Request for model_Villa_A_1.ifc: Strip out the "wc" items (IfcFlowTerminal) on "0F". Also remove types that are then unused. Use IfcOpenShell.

First a look at what the model holds.

```python
import ifcopenshell
import ifcopenshell.util.element

model = ifcopenshell.open("model_Villa_A_1.ifc")
print(model.schema)
storey = next(s for s in model.by_type("IfcBuildingStorey") if s.Name == "0F")
terminals = [e for e in ifcopenshell.util.element.get_decomposition(storey) if e.is_a("IfcFlowTerminal")]
seen = {}
for e in terminals:
    element_type = ifcopenshell.util.element.get_type(e)
    name = element_type.Name if element_type not in (None, e) else None
    seen[name] = seen.get(name, 0) + 1
for name, count in sorted(seen.items(), key=str):
    print(count, "x", name)
```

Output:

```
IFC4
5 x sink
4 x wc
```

```python
import ifcopenshell
import ifcopenshell.api.root
import ifcopenshell.util.element

model = ifcopenshell.open("model_Villa_A_1.ifc")

storey = next(s for s in model.by_type("IfcBuildingStorey") if s.Name == "0F")
terminals = [e for e in ifcopenshell.util.element.get_decomposition(storey) if e.is_a("IfcFlowTerminal")]
targets = [e for e in terminals if (t := ifcopenshell.util.element.get_type(e)) not in (None, e) and t.Name == "wc"]
types = {ifcopenshell.util.element.get_type(e) for e in targets} - {None, *targets}

for e in targets:
    ifcopenshell.api.root.remove_product(model, product=e)
print(len(targets), "removed")

unused = [t for t in types if not ifcopenshell.util.element.get_types(t)]
for t in unused:
    ifcopenshell.api.root.remove_product(model, product=t)
print(len(unused), "unused types removed")

model.write("model_Villa_A_1_updated.ifc")
```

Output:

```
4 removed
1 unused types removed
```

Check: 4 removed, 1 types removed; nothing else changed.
